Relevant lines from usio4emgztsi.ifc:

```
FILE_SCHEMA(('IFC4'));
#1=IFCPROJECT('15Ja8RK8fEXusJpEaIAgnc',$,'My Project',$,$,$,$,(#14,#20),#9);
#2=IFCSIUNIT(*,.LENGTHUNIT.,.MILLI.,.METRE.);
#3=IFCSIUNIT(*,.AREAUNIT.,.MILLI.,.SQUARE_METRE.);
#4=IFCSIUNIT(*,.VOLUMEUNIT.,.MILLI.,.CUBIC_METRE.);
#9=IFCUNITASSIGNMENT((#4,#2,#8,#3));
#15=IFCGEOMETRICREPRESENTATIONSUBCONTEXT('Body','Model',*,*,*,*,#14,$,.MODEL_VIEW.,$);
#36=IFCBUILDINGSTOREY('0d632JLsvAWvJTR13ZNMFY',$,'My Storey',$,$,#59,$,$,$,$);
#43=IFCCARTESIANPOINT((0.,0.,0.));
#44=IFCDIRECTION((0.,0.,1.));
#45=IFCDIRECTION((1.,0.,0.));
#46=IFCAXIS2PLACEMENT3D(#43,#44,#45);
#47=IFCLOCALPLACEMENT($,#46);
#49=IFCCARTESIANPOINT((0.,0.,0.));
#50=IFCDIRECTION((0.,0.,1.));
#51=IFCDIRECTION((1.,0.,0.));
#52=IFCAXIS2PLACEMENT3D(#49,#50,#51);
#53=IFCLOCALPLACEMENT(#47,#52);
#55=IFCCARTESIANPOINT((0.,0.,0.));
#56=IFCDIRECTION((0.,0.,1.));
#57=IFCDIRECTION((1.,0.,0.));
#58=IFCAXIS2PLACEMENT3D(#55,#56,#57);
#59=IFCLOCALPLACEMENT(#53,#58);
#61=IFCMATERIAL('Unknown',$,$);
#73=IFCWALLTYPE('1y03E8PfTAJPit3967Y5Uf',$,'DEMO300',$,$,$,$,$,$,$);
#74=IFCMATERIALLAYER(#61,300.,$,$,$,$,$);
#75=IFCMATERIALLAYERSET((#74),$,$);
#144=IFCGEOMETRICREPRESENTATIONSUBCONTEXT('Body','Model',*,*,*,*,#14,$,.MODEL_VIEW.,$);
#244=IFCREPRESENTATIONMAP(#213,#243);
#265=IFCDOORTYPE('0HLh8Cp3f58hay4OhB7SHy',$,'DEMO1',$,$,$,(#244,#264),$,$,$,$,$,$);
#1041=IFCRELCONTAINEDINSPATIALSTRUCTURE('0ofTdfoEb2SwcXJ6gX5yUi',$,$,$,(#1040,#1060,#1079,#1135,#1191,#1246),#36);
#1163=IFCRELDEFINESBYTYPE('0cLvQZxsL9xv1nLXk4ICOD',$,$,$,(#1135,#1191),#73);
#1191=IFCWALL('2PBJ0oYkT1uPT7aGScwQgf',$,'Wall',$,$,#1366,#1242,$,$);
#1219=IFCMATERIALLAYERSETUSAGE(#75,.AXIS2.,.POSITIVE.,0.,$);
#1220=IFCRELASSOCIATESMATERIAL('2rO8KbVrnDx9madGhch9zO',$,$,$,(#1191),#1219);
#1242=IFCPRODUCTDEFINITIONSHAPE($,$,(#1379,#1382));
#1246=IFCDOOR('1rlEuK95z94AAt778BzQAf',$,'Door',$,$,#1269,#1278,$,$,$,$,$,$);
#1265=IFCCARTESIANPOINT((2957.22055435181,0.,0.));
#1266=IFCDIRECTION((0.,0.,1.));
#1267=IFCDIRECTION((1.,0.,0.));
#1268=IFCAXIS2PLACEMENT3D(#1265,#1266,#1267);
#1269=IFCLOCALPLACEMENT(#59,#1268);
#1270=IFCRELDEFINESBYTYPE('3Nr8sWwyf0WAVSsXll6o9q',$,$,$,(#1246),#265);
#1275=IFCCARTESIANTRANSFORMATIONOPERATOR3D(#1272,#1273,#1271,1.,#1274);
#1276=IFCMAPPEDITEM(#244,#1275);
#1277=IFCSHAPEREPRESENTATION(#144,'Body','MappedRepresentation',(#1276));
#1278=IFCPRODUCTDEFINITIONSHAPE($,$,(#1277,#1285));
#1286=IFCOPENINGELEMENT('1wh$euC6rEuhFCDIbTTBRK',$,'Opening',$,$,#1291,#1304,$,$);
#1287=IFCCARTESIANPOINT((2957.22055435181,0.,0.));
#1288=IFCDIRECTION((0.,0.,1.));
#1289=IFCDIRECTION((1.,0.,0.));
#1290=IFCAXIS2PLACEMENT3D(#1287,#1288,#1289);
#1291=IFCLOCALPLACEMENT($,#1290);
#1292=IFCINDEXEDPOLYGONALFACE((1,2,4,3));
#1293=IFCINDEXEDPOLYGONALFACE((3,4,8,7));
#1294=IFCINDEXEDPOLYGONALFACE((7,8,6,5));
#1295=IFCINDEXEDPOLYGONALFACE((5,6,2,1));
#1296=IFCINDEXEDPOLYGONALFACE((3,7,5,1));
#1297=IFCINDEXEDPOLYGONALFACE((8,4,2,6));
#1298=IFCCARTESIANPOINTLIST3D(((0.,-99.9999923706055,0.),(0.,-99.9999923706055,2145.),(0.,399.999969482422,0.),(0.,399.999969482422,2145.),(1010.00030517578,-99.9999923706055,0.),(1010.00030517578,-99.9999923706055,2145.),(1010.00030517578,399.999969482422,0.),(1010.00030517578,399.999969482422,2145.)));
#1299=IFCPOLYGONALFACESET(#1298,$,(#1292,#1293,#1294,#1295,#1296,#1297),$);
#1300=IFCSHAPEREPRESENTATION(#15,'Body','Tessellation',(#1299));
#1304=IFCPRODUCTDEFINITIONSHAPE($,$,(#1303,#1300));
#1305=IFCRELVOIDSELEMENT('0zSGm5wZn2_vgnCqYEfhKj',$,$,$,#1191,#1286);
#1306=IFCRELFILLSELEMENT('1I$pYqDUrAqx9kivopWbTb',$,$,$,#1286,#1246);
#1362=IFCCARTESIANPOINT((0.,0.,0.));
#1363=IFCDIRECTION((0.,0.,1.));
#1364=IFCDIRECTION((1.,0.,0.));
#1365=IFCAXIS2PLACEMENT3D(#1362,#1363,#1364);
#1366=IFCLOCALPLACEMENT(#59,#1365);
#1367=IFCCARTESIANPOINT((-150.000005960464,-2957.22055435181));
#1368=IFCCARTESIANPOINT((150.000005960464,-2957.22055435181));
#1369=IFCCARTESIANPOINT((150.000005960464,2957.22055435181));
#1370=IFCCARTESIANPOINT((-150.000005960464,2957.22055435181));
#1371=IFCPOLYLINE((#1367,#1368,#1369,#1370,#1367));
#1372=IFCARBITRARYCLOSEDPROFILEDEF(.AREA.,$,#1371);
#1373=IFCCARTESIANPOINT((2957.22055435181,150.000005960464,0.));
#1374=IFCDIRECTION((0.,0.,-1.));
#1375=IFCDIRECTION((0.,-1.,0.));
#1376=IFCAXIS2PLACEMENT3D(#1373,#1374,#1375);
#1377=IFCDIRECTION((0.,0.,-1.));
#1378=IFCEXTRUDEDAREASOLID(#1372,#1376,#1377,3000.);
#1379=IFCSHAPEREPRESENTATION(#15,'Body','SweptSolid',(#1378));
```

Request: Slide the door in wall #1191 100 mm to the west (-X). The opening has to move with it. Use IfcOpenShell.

```python
import ifcopenshell
import ifcopenshell.api.geometry
import ifcopenshell.util.placement
import ifcopenshell.util.unit

model = ifcopenshell.open("usio4emgztsi.ifc")
unit_scale = ifcopenshell.util.unit.calculate_unit_scale(model)

door = model.by_guid("1rlEuK95z94AAt778BzQAf")
opening = door.FillsVoids[0].RelatingOpeningElement
wall = opening.VoidsElements[0].RelatingBuildingElement

wall_matrix = ifcopenshell.util.placement.get_local_placement(wall.ObjectPlacement)
shift = wall_matrix[:3, 0] * -0.1 / unit_scale
before = ifcopenshell.util.placement.get_local_placement(door.ObjectPlacement)[:3, 3].copy()

# The door is not placed relative to its opening, so move both.
for product in (opening, door):
    matrix = ifcopenshell.util.placement.get_local_placement(product.ObjectPlacement)
    matrix[:3, 3] += shift
    ifcopenshell.api.geometry.edit_object_placement(model, product=product, matrix=matrix, is_si=False)

after = ifcopenshell.util.placement.get_local_placement(door.ObjectPlacement)[:3, 3]
print("door moved by", (after - before).round(3) + 0.0)

model.write("usio4emgztsi_updated.ifc")
```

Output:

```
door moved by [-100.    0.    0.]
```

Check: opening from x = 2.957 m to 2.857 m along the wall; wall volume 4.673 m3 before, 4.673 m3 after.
